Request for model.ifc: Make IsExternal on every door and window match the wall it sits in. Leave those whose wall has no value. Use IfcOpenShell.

First a look at what the model holds.

```python
import ifcopenshell
import ifcopenshell.util.element

model = ifcopenshell.open("model.ifc")
print(model.schema)
seen = {}
for e in model.by_type("IfcDoor") + model.by_type("IfcWindow"):
    if not e.FillsVoids:
        continue
    host = e.FillsVoids[0].RelatingOpeningElement.VoidsElements[0].RelatingBuildingElement
    own = ifcopenshell.util.element.get_pset(e, f"Pset_{e.is_a()[3:].removesuffix('StandardCase')}Common", "IsExternal")
    wall = ifcopenshell.util.element.get_pset(host, "Pset_WallCommon", "IsExternal")
    seen[e.is_a(), own, wall] = seen.get((e.is_a(), own, wall), 0) + 1
for (cls, own, wall), count in sorted(seen.items(), key=str):
    print(count, cls, "IsExternal:", own, "| host wall:", wall)
```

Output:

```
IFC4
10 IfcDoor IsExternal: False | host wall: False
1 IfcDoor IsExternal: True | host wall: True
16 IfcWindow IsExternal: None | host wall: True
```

```python
import ifcopenshell
import ifcopenshell.api.pset
import ifcopenshell.util.element

model = ifcopenshell.open("model.ifc")

count = 0
for ifc_class, pset_name in (("IfcDoor", "Pset_DoorCommon"), ("IfcWindow", "Pset_WindowCommon")):
    for e in model.by_type(ifc_class):
        if not e.FillsVoids:
            continue
        host = e.FillsVoids[0].RelatingOpeningElement.VoidsElements[0].RelatingBuildingElement
        external = ifcopenshell.util.element.get_pset(host, "Pset_WallCommon", "IsExternal")
        if external is None or ifcopenshell.util.element.get_pset(e, pset_name, "IsExternal") == external:
            continue
        pset = ifcopenshell.api.pset.add_pset(model, product=e, name=pset_name)
        ifcopenshell.api.pset.edit_pset(model, pset=pset, properties={"IsExternal": external})
        count += 1

print(count, "updated")

model.write("model_updated.ifc")
```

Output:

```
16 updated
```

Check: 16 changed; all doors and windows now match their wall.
